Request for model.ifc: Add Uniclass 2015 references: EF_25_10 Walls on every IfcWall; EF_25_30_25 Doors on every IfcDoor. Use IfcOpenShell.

First a look at what the model holds.

```python
import ifcopenshell

model = ifcopenshell.open("model.ifc")
print(model.schema)
print("classifications:", [c.Name for c in model.by_type("IfcClassification")])
for ifc_class in ("IfcDoor", "IfcRoof", "IfcStair", "IfcWall", "IfcWindow"):
    print(ifc_class, len(model.by_type(ifc_class)))
```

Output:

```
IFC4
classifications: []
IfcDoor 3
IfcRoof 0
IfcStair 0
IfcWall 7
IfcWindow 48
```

```python
import ifcopenshell
import ifcopenshell.api.classification

model = ifcopenshell.open("model.ifc")

system = ifcopenshell.api.classification.add_classification(model, classification="Uniclass 2015")

codes = {
    "IfcWall": ("EF_25_10", "Walls"),
    "IfcDoor": ("EF_25_30_25", "Doors"),
}
for ifc_class, (code, name) in codes.items():
    products = model.by_type(ifc_class)
    ifcopenshell.api.classification.add_reference(
        model, products=products, classification=system, identification=code, name=name
    )
    print(code, len(products))

model.write("model-out.ifc")
```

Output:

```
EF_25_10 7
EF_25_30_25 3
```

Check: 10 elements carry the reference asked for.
